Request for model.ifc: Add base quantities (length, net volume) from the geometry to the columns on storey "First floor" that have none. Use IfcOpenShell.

First a look at what the model holds.

```python
import ifcopenshell
import ifcopenshell.util.element
import ifcopenshell.util.unit

model = ifcopenshell.open("model.ifc")
print(model.schema)
for unit_type in ("LENGTHUNIT", "AREAUNIT", "VOLUMEUNIT"):
    print(unit_type, ifcopenshell.util.unit.calculate_unit_scale(model, unit_type))
storey = next(s for s in model.by_type("IfcBuildingStorey") if s.Name == "First floor")
columns = [e for e in ifcopenshell.util.element.get_decomposition(storey) if e.is_a("IfcColumn")]
for e in sorted(columns, key=lambda e: e.id()):
    print(e.id(), e.is_a(), e.Name, list(ifcopenshell.util.element.get_psets(e, qtos_only=True)), sep=" | ")
```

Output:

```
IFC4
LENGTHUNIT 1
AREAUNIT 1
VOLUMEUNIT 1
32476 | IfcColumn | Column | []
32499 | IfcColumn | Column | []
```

```python
import ifcopenshell
import ifcopenshell.api.pset
import ifcopenshell.geom
import ifcopenshell.util.element
import ifcopenshell.util.shape
import ifcopenshell.util.unit

model = ifcopenshell.open("model.ifc")
unit_scale = ifcopenshell.util.unit.calculate_unit_scale(model)
volume_scale = ifcopenshell.util.unit.calculate_unit_scale(model, "VOLUMEUNIT")
settings = ifcopenshell.geom.settings()

storey = next(s for s in model.by_type("IfcBuildingStorey") if s.Name == "First floor")
columns = [e for e in ifcopenshell.util.element.get_decomposition(storey) if e.is_a("IfcColumn")]

for e in sorted(columns, key=lambda e: e.id()):
    if ifcopenshell.util.element.get_psets(e, qtos_only=True, should_inherit=False):
        continue
    # Geometry comes back in metres, in the element's own axes.
    shape = ifcopenshell.geom.create_shape(settings, e)
    values = {
        "Length": ifcopenshell.util.shape.get_z(shape.geometry) / unit_scale,
        "NetVolume": ifcopenshell.util.shape.get_volume(shape.geometry) / volume_scale,
    }
    qto = ifcopenshell.api.pset.add_qto(model, product=e, name="Qto_ColumnBaseQuantities")
    ifcopenshell.api.pset.edit_qto(model, qto=qto, properties=values)
    print(e.id(), {k: round(v, 3) for k, v in values.items()})

model.write("model_updated.ifc")
```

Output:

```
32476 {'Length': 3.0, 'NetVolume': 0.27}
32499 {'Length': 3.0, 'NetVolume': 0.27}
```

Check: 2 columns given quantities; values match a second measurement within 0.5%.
